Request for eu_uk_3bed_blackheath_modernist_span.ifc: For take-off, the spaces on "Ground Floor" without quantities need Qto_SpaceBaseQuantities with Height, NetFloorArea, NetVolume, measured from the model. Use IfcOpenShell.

First a look at what the model holds.

```python
import ifcopenshell
import ifcopenshell.util.element
import ifcopenshell.util.unit

model = ifcopenshell.open("eu_uk_3bed_blackheath_modernist_span.ifc")
print(model.schema)
for unit_type in ("LENGTHUNIT", "AREAUNIT", "VOLUMEUNIT"):
    print(unit_type, ifcopenshell.util.unit.calculate_unit_scale(model, unit_type))
storey = next(s for s in model.by_type("IfcBuildingStorey") if s.Name == "Ground Floor")
spaces = [e for e in ifcopenshell.util.element.get_decomposition(storey) if e.is_a("IfcSpace")]
for e in sorted(spaces, key=lambda e: e.id()):
    print(e.id(), e.is_a(), e.Name, list(ifcopenshell.util.element.get_psets(e, qtos_only=True)), sep=" | ")
```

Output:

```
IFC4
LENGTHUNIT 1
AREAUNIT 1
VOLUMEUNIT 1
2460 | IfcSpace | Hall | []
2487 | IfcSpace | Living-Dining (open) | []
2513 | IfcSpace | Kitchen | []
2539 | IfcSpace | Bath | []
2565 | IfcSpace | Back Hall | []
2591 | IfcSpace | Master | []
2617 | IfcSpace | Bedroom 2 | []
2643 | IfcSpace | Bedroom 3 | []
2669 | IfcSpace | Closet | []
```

```python
import ifcopenshell
import ifcopenshell.api.pset
import ifcopenshell.geom
import ifcopenshell.util.element
import ifcopenshell.util.shape
import ifcopenshell.util.unit

model = ifcopenshell.open("eu_uk_3bed_blackheath_modernist_span.ifc")
unit_scale = ifcopenshell.util.unit.calculate_unit_scale(model)
area_scale = ifcopenshell.util.unit.calculate_unit_scale(model, "AREAUNIT")
volume_scale = ifcopenshell.util.unit.calculate_unit_scale(model, "VOLUMEUNIT")
settings = ifcopenshell.geom.settings()

storey = next(s for s in model.by_type("IfcBuildingStorey") if s.Name == "Ground Floor")
spaces = [e for e in ifcopenshell.util.element.get_decomposition(storey) if e.is_a("IfcSpace")]

for e in sorted(spaces, key=lambda e: e.id()):
    if ifcopenshell.util.element.get_psets(e, qtos_only=True, should_inherit=False):
        continue
    # Geometry comes back in metres, in the element's own axes.
    shape = ifcopenshell.geom.create_shape(settings, e)
    values = {
        "Height": ifcopenshell.util.shape.get_z(shape.geometry) / unit_scale,
        "NetFloorArea": ifcopenshell.util.shape.get_footprint_area(shape.geometry) / area_scale,
        "NetVolume": ifcopenshell.util.shape.get_volume(shape.geometry) / volume_scale,
    }
    qto = ifcopenshell.api.pset.add_qto(model, product=e, name="Qto_SpaceBaseQuantities")
    ifcopenshell.api.pset.edit_qto(model, qto=qto, properties=values)
    print(e.id(), {k: round(v, 3) for k, v in values.items()})

model.write("eu_uk_3bed_blackheath_modernist_span_edited.ifc")
```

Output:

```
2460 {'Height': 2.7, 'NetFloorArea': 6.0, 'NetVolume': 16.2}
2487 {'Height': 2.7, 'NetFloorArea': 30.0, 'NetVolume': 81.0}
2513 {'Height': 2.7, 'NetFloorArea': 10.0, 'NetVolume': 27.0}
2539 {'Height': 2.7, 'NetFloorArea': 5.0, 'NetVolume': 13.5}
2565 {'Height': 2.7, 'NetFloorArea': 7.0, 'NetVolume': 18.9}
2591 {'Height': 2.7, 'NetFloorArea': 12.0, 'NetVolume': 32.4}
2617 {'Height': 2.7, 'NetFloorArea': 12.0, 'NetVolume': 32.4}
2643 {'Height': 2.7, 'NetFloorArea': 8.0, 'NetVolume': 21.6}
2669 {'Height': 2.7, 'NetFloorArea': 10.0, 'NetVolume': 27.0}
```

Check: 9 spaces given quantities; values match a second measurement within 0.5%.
